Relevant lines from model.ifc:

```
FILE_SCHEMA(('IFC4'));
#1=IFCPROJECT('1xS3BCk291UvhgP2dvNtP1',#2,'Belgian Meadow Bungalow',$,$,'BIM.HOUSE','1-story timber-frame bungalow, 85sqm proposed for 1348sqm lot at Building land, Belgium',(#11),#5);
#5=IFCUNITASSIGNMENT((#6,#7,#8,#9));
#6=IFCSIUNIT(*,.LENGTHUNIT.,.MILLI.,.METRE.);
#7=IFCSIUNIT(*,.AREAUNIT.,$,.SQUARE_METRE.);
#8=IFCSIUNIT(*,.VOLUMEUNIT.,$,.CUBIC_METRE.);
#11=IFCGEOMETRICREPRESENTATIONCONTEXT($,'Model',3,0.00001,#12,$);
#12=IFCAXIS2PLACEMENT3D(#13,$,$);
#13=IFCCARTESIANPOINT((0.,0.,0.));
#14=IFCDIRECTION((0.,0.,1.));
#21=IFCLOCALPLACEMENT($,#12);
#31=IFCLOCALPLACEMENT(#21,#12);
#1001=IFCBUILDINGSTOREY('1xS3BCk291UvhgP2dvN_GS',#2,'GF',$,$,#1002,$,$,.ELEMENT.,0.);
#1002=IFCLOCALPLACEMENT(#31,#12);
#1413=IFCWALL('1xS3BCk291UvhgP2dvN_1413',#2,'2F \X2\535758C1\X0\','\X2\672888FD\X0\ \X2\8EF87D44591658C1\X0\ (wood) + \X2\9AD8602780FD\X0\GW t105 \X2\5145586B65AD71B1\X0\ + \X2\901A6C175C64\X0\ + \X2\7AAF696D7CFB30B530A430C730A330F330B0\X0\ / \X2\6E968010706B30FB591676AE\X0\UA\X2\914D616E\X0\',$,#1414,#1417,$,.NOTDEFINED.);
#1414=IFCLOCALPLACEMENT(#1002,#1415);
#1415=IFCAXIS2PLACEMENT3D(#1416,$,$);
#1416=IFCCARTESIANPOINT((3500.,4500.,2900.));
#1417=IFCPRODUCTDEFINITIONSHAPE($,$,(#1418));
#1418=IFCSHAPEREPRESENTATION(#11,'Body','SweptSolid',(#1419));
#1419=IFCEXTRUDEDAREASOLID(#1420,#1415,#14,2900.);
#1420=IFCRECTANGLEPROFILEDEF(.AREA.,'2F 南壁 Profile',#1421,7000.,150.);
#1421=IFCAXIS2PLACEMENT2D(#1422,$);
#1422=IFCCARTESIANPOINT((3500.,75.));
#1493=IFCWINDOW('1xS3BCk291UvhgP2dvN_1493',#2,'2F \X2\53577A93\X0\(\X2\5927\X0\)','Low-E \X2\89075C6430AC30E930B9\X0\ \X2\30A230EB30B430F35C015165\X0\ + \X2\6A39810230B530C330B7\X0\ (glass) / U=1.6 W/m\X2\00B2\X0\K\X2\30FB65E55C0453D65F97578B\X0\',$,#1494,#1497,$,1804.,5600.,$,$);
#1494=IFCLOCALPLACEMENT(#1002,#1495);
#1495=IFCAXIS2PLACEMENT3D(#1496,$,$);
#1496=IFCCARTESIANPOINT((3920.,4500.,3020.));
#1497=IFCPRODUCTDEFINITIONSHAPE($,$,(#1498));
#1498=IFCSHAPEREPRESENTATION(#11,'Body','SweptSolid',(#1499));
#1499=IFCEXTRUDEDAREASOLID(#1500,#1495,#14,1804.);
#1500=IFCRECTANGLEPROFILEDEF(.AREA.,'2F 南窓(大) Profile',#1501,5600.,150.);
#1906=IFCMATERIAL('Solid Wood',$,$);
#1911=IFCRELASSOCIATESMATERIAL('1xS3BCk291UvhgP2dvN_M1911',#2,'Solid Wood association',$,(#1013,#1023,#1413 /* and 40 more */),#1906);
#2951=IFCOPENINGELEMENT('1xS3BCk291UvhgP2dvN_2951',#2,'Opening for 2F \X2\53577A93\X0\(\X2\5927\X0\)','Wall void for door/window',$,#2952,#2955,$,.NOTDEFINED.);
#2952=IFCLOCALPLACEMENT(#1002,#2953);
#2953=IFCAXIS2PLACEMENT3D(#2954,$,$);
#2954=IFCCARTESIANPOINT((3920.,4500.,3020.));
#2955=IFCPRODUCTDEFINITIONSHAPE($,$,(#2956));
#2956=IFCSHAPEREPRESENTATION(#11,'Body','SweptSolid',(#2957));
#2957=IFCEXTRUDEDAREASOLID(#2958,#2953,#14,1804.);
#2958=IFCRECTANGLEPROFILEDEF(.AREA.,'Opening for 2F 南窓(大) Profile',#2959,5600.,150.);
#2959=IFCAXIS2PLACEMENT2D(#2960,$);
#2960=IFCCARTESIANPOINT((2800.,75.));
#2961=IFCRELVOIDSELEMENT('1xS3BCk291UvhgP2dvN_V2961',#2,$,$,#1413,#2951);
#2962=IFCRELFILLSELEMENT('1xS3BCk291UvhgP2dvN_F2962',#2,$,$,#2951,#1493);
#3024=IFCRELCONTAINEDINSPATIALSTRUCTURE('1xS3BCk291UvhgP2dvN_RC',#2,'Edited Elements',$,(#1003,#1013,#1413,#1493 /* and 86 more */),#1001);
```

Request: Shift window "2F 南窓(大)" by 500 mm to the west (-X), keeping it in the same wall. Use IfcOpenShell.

```python
import ifcopenshell
import ifcopenshell.api.geometry
import ifcopenshell.util.placement
import ifcopenshell.util.unit

model = ifcopenshell.open("model.ifc")
unit_scale = ifcopenshell.util.unit.calculate_unit_scale(model)

window = model.by_guid("1xS3BCk291UvhgP2dvN_1493")
opening = window.FillsVoids[0].RelatingOpeningElement
wall = opening.VoidsElements[0].RelatingBuildingElement

wall_matrix = ifcopenshell.util.placement.get_local_placement(wall.ObjectPlacement)
shift = wall_matrix[:3, 0] * -0.5 / unit_scale
before = ifcopenshell.util.placement.get_local_placement(window.ObjectPlacement)[:3, 3].copy()

# The window is not placed relative to its opening, so move both.
for product in (opening, window):
    matrix = ifcopenshell.util.placement.get_local_placement(product.ObjectPlacement)
    matrix[:3, 3] += shift
    ifcopenshell.api.geometry.edit_object_placement(model, product=product, matrix=matrix, is_si=False)

after = ifcopenshell.util.placement.get_local_placement(window.ObjectPlacement)[:3, 3]
print("window moved by", (after - before).round(3) + 0.0)

model.write("model-out.ifc")
```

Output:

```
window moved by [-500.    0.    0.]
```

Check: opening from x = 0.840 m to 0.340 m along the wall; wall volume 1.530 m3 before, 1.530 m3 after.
